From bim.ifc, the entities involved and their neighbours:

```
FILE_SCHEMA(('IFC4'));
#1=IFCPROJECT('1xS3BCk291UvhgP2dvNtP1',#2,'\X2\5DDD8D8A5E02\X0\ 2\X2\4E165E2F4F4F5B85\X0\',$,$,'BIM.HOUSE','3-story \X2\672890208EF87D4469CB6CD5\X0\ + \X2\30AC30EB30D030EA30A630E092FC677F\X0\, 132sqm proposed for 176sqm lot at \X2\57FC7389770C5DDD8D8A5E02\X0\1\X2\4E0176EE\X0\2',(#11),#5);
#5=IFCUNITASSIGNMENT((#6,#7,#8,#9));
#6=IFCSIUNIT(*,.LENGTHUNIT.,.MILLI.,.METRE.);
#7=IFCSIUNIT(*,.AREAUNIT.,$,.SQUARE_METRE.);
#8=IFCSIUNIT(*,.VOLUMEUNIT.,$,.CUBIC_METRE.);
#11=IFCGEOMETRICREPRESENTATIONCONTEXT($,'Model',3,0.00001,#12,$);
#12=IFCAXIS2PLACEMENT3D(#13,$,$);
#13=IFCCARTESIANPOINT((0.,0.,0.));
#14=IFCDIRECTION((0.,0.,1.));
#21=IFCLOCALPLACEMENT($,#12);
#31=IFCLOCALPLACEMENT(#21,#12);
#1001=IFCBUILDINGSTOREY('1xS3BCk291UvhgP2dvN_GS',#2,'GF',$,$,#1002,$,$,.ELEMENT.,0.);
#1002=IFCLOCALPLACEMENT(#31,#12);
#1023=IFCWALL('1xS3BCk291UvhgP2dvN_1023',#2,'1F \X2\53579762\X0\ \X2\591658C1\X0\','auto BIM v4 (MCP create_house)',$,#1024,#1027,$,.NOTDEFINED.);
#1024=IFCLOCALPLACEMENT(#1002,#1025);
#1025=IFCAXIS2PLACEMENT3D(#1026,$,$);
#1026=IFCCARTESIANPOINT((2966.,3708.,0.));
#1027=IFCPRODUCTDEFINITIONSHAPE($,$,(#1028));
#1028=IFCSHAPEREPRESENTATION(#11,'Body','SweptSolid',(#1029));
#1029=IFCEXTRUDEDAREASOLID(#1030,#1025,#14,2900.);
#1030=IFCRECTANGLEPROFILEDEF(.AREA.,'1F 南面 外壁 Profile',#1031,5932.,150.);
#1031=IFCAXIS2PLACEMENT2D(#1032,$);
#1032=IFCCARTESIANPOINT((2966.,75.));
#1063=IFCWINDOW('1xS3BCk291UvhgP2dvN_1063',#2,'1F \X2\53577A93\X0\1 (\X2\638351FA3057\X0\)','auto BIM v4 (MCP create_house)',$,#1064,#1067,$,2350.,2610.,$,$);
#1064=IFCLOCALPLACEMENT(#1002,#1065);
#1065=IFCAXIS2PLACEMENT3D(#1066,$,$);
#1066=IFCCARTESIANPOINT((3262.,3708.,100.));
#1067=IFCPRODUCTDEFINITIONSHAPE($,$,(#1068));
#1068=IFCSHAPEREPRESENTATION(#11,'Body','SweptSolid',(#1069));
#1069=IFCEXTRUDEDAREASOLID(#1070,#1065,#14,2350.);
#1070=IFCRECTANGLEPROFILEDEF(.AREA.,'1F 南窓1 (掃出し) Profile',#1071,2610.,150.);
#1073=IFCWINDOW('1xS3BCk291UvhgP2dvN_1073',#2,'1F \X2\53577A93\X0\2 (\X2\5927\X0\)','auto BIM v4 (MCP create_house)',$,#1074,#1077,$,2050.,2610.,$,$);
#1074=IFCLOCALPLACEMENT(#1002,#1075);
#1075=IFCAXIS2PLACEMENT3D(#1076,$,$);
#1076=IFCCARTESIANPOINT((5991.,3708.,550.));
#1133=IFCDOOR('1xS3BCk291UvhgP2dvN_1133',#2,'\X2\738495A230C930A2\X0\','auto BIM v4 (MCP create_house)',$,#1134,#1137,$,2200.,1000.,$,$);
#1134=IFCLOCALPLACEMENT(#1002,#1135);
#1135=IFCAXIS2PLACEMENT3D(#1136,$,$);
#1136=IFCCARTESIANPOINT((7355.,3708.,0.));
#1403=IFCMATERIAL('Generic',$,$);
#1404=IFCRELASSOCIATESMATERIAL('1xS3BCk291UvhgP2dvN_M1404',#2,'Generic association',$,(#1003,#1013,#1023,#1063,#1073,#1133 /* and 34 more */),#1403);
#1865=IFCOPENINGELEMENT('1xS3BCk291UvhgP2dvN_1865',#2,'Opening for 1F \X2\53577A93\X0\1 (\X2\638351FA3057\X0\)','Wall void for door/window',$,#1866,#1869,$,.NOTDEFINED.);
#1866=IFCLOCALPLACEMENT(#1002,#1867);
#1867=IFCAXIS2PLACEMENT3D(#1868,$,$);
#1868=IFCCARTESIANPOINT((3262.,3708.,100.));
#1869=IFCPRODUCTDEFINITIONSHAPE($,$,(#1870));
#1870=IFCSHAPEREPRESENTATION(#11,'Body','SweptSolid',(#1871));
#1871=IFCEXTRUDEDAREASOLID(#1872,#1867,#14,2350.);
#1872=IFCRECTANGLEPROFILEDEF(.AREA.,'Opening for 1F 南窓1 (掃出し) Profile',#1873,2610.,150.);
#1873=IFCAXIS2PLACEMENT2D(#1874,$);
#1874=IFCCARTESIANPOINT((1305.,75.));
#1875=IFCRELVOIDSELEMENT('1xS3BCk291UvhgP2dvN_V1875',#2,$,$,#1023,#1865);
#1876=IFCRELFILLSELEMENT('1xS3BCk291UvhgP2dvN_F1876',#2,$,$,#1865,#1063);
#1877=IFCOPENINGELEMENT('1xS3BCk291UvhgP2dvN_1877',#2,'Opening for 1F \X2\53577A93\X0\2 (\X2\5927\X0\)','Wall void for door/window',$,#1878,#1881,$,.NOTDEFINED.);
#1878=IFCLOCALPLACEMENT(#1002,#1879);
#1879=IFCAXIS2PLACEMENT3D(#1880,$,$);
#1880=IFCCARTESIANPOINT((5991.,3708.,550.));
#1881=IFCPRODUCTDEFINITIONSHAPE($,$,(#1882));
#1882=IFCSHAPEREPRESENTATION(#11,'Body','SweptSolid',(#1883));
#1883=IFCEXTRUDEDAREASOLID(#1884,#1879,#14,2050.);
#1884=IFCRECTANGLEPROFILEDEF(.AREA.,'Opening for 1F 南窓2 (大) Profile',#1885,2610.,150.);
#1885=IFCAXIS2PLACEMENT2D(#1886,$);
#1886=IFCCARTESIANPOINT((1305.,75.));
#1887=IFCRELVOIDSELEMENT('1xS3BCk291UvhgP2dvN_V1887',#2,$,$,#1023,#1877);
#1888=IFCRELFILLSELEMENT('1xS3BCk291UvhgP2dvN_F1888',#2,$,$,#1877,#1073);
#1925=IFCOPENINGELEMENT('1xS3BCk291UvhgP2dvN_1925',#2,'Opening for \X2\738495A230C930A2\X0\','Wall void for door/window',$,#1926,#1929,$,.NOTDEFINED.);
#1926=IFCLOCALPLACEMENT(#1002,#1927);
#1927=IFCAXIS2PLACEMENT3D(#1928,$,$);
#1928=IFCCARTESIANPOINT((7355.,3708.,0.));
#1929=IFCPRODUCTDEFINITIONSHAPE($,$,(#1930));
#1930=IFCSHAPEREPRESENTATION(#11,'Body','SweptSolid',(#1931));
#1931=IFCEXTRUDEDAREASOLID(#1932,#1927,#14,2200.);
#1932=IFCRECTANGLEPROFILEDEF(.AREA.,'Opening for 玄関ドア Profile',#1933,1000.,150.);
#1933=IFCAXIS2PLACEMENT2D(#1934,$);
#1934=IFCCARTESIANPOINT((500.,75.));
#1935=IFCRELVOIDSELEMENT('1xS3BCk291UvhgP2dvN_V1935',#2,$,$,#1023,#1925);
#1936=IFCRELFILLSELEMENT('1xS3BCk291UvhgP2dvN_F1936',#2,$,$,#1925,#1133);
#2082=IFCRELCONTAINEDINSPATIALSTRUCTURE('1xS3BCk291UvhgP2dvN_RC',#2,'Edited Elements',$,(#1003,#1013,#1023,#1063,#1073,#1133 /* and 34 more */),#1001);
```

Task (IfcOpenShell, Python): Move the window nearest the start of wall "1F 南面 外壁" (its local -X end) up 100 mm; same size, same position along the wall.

```python
import numpy as np
import ifcopenshell
import ifcopenshell.api.geometry
import ifcopenshell.util.placement
import ifcopenshell.util.unit

model = ifcopenshell.open("bim.ifc")
unit_scale = ifcopenshell.util.unit.calculate_unit_scale(model)

window = model.by_guid("1xS3BCk291UvhgP2dvN_1063")
opening = window.FillsVoids[0].RelatingOpeningElement
dz = 0.1 / unit_scale

shift = np.array([0.0, 0.0, dz])
# The window is not placed relative to its opening, so move both.
for product in (opening, window):
    matrix = ifcopenshell.util.placement.get_local_placement(product.ObjectPlacement)
    matrix[:3, 3] += shift
    ifcopenshell.api.geometry.edit_object_placement(model, product=product, matrix=matrix, is_si=False)

print(f"moved by {dz * unit_scale:+.3f} m")

model.write("bim_rev.ifc")
```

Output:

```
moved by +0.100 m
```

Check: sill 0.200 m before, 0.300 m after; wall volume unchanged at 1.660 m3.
